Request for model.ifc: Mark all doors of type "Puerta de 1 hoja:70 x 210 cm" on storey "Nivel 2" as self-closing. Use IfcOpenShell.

First a look at what the model holds.

```python
import ifcopenshell
import ifcopenshell.util.element

model = ifcopenshell.open("model.ifc")
print(model.schema)
storey = next(s for s in model.by_type("IfcBuildingStorey") if s.Name == "Nivel 2")
doors = [e for e in ifcopenshell.util.element.get_decomposition(storey) if e.is_a("IfcDoor")]
seen = {}
for e in doors:
    element_type = ifcopenshell.util.element.get_type(e)
    key = (element_type.Name if element_type != e and element_type else None, ifcopenshell.util.element.get_pset(e, "Pset_DoorCommon", "SelfClosing"))
    seen[key] = seen.get(key, 0) + 1
for (name, value), count in sorted(seen.items(), key=str):
    print(count, "x", name, "|", value)
```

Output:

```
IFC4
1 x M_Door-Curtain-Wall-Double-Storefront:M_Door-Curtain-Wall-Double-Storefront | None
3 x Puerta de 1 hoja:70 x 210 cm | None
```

```python
import ifcopenshell
import ifcopenshell.api.pset
import ifcopenshell.util.element

model = ifcopenshell.open("model.ifc")

storey = next(s for s in model.by_type("IfcBuildingStorey") if s.Name == "Nivel 2")
doors = [e for e in ifcopenshell.util.element.get_decomposition(storey) if e.is_a("IfcDoor")]

count = 0
for e in doors:
    element_type = ifcopenshell.util.element.get_type(e)
    if element_type in (None, e) or element_type.Name != "Puerta de 1 hoja:70 x 210 cm":
        continue
    # add_pset returns the element's existing set when there is one.
    pset = ifcopenshell.api.pset.add_pset(model, product=e, name="Pset_DoorCommon")
    ifcopenshell.api.pset.edit_pset(model, pset=pset, properties={"SelfClosing": True})
    count += 1

print(count, "doors updated")

model.write("model_v2.ifc")
```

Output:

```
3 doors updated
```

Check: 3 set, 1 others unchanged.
